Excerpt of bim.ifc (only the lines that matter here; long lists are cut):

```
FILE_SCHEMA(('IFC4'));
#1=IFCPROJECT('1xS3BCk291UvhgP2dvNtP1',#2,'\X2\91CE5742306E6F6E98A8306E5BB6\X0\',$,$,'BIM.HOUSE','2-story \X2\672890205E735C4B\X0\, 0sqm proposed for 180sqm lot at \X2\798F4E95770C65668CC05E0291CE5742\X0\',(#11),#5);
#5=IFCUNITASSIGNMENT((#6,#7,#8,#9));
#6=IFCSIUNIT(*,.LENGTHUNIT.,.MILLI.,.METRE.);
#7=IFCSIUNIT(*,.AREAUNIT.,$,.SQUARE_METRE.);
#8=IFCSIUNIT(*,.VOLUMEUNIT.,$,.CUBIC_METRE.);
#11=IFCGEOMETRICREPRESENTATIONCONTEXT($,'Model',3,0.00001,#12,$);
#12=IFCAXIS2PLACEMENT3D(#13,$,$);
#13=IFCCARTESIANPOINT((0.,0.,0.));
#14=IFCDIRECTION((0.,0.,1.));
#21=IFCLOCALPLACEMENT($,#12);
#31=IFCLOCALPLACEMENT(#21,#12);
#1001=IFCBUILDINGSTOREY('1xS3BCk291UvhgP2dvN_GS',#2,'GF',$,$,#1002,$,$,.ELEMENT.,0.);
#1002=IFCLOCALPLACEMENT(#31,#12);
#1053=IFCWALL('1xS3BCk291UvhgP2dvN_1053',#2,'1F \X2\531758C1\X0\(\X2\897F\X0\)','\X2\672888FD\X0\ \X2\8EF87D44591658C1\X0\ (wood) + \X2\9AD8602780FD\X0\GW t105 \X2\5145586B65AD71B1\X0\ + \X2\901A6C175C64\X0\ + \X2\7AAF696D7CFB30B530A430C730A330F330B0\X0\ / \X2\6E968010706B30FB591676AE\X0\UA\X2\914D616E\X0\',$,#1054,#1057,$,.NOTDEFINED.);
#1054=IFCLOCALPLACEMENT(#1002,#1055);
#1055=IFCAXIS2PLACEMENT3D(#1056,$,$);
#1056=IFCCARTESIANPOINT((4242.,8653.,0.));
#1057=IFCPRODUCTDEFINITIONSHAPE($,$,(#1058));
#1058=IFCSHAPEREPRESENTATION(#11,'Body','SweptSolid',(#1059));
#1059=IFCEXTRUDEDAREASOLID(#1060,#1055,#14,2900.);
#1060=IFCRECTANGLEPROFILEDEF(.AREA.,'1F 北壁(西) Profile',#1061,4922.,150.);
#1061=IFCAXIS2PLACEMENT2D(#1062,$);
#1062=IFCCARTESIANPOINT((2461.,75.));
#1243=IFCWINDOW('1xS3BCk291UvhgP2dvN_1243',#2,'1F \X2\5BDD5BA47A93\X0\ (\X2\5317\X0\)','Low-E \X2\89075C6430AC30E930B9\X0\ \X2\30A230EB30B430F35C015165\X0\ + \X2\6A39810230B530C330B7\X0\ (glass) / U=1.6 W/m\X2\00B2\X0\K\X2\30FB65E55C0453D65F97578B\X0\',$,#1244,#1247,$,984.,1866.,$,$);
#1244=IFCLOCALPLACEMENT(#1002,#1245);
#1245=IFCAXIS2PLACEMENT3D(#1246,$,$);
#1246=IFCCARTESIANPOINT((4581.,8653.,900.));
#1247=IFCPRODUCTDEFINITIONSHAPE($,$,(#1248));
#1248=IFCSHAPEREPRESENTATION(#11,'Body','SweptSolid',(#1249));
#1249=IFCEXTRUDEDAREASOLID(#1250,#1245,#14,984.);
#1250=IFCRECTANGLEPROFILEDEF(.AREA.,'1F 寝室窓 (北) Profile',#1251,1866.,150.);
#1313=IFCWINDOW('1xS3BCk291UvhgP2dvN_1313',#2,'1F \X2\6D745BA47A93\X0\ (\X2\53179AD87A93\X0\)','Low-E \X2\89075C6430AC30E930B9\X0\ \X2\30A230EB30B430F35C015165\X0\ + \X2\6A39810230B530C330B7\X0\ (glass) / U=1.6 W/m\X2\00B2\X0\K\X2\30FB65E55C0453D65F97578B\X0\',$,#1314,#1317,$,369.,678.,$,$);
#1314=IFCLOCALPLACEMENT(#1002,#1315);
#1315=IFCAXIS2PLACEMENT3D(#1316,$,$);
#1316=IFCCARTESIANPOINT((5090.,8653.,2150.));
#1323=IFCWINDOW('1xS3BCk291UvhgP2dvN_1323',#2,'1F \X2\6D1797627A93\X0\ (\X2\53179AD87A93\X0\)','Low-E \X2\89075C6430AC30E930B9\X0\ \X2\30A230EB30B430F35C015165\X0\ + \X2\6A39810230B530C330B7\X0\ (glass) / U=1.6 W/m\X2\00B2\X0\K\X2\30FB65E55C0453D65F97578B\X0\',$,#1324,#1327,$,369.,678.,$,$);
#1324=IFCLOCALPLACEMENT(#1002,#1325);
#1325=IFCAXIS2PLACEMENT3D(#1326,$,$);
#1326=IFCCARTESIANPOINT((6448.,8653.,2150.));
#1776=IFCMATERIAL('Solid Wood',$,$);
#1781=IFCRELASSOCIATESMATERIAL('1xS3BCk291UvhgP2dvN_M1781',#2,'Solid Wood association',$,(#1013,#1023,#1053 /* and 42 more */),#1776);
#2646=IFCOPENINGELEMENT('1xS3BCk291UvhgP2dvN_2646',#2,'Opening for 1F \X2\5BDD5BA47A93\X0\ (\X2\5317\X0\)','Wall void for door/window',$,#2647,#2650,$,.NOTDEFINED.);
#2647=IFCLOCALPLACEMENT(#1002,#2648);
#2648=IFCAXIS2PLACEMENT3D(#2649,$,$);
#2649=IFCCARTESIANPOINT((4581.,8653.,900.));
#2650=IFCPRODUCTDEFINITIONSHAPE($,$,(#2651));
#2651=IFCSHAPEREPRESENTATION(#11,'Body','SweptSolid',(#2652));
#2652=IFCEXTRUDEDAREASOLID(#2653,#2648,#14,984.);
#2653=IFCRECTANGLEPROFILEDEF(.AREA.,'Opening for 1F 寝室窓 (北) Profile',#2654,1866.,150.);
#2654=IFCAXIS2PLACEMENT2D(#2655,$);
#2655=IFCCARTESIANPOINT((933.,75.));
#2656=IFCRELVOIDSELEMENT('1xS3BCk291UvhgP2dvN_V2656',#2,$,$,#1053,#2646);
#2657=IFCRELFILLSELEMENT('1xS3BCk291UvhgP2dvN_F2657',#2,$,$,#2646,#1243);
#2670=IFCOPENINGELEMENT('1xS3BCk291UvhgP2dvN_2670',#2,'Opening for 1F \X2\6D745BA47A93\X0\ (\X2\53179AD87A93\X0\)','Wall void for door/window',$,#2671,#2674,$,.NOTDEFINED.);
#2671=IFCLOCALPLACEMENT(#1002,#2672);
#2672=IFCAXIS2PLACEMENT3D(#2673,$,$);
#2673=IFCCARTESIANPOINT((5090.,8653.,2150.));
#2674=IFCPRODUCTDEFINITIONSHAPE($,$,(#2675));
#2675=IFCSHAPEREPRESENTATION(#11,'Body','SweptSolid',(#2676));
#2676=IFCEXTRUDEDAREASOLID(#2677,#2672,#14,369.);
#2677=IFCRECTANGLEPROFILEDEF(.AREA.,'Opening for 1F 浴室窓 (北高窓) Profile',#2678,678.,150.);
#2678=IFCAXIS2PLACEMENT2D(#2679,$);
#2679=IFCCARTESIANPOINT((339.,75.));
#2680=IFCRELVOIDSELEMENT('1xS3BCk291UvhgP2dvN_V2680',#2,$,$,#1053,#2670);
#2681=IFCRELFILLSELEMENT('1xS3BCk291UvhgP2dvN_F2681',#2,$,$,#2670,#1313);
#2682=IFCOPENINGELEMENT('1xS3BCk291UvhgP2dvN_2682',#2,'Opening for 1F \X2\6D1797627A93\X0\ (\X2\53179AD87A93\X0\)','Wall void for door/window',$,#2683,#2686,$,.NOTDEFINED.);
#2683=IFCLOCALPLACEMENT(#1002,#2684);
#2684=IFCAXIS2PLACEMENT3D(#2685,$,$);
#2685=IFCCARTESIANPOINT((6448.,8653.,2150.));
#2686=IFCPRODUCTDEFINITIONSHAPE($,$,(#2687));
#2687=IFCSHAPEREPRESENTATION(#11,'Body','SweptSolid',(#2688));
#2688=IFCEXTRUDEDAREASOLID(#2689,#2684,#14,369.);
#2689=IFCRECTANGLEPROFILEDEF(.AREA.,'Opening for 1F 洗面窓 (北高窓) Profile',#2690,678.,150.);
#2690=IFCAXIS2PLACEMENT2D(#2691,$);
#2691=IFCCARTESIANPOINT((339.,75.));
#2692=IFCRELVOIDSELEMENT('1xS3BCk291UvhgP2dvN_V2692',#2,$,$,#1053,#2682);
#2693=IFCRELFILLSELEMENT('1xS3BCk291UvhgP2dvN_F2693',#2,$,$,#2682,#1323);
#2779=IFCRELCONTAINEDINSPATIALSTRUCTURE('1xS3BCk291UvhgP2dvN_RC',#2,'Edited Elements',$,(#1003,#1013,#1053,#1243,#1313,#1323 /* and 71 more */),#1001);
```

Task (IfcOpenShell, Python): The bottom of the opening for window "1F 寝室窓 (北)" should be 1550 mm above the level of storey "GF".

```python
import numpy as np
import ifcopenshell
import ifcopenshell.api.geometry
import ifcopenshell.geom
import ifcopenshell.util.element
import ifcopenshell.util.placement
import ifcopenshell.util.shape
import ifcopenshell.util.unit

model = ifcopenshell.open("bim.ifc")
unit_scale = ifcopenshell.util.unit.calculate_unit_scale(model)

window = model.by_guid("1xS3BCk291UvhgP2dvN_1243")
opening = window.FillsVoids[0].RelatingOpeningElement
storey = ifcopenshell.util.element.get_container(window, ifc_class="IfcBuildingStorey")
level = ifcopenshell.util.placement.get_local_placement(storey.ObjectPlacement)[2, 3]

# The opening's origin need not be at the sill, so measure its lowest point.
shape = ifcopenshell.geom.create_shape(ifcopenshell.geom.settings(), opening)
bottom = ifcopenshell.util.shape.get_shape_bottom_elevation(shape, shape.geometry) / unit_scale
dz = level + 1550.0 - bottom

shift = np.array([0.0, 0.0, dz])
# The window is not placed relative to its opening, so move both.
for product in (opening, window):
    matrix = ifcopenshell.util.placement.get_local_placement(product.ObjectPlacement)
    matrix[:3, 3] += shift
    ifcopenshell.api.geometry.edit_object_placement(model, product=product, matrix=matrix, is_si=False)

print(f"moved by {dz * unit_scale:+.3f} m")

model.write("bim_edited.ifc")
```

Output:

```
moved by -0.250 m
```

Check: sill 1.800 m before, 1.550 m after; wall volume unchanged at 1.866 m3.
